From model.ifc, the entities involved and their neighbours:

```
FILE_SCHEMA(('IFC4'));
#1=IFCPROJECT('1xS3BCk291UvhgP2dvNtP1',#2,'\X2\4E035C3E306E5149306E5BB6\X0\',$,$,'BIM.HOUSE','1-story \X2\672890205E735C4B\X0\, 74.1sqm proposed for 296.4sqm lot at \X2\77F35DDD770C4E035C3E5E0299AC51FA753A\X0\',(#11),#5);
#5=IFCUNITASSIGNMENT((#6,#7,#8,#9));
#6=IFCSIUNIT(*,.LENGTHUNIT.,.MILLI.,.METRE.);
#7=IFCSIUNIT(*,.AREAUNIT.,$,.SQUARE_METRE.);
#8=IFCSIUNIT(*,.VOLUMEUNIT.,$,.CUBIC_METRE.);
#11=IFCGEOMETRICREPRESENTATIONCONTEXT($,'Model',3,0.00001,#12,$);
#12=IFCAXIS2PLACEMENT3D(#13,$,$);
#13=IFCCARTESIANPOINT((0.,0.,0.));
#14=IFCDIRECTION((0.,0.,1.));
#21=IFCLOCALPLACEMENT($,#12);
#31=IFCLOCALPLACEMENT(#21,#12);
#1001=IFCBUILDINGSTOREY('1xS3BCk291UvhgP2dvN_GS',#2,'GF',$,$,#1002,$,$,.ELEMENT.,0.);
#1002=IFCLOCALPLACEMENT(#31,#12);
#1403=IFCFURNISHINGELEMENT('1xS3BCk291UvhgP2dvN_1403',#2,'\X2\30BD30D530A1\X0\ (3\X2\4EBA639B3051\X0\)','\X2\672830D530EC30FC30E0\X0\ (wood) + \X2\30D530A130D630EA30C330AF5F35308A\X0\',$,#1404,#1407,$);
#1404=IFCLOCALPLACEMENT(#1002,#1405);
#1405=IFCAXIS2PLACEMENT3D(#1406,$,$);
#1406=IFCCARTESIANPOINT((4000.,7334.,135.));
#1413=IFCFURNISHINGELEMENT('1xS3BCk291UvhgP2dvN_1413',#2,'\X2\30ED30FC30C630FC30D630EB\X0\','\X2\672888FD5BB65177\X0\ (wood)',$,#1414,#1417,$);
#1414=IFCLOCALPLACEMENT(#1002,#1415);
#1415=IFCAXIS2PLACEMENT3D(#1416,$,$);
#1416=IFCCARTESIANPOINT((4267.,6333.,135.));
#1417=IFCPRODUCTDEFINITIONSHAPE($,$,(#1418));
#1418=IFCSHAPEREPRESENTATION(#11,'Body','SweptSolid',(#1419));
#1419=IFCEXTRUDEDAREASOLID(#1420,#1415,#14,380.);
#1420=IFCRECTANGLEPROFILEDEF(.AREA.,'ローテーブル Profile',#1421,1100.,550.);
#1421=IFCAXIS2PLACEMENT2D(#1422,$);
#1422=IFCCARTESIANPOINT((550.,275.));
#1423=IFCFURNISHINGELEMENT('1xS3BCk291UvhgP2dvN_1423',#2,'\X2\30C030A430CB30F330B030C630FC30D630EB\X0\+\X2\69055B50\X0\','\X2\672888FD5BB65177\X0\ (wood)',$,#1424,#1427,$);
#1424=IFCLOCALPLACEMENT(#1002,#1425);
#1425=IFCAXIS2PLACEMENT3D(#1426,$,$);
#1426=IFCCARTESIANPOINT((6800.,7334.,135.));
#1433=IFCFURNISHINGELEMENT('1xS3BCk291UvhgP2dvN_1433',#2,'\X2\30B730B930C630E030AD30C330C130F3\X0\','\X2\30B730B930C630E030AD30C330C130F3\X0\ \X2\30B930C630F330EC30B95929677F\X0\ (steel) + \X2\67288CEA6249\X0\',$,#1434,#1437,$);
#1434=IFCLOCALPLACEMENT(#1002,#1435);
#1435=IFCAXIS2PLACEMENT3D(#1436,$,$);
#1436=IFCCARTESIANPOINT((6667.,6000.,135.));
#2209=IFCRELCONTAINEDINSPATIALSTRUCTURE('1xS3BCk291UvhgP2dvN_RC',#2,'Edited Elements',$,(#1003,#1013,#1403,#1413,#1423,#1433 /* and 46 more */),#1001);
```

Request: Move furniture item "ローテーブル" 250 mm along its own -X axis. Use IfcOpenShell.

```python
import ifcopenshell
import ifcopenshell.api.geometry
import ifcopenshell.util.placement
import ifcopenshell.util.unit

model = ifcopenshell.open("model.ifc")
unit_scale = ifcopenshell.util.unit.calculate_unit_scale(model)

item = model.by_guid("1xS3BCk291UvhgP2dvN_1413")
matrix = ifcopenshell.util.placement.get_local_placement(item.ObjectPlacement)
matrix[:3, 3] -= matrix[:3, 0] * 0.25 / unit_scale
ifcopenshell.api.geometry.edit_object_placement(model, product=item, matrix=matrix, is_si=False)

print(ifcopenshell.util.placement.get_local_placement(item.ObjectPlacement).round(3) + 0.0)

model.write("model_rev.ifc")
```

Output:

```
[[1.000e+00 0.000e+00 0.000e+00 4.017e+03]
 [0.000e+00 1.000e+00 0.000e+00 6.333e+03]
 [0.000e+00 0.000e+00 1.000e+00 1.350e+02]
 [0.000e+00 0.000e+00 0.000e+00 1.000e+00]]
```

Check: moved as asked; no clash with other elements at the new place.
